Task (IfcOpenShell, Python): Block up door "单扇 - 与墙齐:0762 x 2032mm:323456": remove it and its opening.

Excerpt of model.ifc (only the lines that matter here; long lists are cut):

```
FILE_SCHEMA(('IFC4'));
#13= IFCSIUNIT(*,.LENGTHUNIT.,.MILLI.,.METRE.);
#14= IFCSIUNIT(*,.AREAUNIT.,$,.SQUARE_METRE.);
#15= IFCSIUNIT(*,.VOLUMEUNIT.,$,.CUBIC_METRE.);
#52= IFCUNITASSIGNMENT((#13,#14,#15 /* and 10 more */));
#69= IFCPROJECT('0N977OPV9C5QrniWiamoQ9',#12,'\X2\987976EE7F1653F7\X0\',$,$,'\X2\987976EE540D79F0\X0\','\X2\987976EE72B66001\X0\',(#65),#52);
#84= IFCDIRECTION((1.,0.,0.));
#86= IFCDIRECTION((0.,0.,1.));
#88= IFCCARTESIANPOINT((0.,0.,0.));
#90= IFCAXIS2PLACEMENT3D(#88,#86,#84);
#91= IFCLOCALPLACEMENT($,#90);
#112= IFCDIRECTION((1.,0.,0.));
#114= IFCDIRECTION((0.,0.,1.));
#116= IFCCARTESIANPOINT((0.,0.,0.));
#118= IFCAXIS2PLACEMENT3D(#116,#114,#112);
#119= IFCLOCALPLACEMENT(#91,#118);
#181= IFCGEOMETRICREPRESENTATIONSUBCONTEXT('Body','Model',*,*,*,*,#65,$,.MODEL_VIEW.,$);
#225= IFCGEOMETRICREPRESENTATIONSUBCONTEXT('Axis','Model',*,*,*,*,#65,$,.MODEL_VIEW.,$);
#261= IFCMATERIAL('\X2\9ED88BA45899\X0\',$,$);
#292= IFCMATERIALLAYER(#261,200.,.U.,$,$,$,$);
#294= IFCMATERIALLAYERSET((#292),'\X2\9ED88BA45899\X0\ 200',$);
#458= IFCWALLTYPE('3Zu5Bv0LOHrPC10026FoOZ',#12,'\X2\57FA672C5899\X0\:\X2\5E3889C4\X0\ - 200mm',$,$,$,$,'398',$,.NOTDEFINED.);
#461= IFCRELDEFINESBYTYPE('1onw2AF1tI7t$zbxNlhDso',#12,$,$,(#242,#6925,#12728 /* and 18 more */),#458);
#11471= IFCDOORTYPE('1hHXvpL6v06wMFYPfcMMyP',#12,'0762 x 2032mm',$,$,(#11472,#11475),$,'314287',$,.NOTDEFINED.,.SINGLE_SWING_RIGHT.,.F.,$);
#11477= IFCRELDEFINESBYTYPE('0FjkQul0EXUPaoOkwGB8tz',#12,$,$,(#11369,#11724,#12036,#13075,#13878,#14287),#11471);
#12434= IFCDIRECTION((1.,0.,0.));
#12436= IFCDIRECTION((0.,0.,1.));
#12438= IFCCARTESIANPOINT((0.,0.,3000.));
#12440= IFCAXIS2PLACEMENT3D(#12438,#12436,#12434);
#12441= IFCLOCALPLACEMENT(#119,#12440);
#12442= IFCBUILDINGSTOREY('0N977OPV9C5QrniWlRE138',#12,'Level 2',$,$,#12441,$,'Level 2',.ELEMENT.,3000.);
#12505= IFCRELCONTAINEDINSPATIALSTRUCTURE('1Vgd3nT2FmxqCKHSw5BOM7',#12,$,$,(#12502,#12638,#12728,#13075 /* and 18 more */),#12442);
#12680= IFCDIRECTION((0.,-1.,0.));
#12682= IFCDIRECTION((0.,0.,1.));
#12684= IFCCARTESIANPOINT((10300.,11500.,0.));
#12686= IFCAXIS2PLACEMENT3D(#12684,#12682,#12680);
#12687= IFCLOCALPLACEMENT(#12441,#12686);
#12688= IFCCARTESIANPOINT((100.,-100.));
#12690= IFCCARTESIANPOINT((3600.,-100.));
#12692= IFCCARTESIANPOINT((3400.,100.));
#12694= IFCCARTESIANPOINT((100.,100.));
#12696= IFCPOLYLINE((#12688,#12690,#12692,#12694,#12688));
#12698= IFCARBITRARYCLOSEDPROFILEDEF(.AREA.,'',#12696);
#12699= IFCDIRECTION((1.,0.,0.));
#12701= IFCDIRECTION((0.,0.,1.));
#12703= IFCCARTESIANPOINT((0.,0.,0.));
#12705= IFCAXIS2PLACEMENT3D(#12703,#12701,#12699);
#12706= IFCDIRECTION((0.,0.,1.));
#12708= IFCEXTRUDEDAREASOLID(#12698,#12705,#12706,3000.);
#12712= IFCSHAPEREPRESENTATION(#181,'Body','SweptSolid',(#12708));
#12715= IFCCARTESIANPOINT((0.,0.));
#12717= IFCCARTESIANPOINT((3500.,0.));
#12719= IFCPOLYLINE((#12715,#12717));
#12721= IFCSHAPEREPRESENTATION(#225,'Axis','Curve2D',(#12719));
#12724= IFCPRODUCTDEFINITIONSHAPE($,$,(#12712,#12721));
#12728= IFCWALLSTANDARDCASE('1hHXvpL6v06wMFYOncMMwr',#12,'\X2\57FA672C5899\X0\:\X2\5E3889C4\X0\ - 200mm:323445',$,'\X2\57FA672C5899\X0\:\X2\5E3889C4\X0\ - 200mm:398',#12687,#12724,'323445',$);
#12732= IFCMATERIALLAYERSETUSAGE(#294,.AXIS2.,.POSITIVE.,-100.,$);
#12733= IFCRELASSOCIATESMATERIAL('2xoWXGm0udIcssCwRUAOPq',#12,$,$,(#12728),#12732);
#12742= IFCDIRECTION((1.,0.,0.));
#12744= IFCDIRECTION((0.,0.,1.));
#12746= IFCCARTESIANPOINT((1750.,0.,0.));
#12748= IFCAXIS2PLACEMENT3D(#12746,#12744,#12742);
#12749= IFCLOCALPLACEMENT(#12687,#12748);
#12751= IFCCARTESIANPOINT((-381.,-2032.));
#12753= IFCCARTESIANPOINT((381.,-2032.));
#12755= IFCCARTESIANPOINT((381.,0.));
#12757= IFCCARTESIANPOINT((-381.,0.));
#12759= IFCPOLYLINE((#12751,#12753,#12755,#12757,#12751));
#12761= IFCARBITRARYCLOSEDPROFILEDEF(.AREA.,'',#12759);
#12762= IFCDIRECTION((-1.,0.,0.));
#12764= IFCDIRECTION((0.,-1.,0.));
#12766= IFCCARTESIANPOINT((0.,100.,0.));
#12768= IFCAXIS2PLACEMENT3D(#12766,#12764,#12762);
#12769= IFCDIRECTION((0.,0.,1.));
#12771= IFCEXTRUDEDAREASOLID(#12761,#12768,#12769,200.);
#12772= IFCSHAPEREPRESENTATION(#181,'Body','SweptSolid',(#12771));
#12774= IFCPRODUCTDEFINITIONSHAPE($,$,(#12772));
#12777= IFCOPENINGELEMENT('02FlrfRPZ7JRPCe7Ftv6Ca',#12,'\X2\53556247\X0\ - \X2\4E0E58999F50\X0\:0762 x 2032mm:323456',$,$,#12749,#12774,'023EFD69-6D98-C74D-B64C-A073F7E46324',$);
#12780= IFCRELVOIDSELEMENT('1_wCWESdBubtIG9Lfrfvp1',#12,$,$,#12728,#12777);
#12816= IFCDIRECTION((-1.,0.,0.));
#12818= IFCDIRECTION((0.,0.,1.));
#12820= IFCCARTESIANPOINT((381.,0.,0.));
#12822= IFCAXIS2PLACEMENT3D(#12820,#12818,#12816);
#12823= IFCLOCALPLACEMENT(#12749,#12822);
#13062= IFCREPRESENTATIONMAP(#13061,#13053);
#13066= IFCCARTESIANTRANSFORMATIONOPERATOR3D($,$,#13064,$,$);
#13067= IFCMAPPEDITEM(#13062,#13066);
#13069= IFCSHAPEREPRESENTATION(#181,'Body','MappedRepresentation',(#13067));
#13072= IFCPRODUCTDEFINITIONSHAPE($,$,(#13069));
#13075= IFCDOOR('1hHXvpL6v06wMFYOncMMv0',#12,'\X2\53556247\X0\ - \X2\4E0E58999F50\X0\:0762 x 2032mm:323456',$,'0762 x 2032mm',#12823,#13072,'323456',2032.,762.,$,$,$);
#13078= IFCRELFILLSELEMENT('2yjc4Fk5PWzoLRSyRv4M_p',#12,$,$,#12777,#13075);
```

```python
import ifcopenshell
import ifcopenshell.api.feature
import ifcopenshell.api.root
import ifcopenshell.geom
import ifcopenshell.util.shape

model = ifcopenshell.open("model.ifc")
settings = ifcopenshell.geom.settings()


def volume(element):
    """Net volume in cubic metres, openings subtracted."""
    shape = ifcopenshell.geom.create_shape(settings, element)
    return ifcopenshell.util.shape.get_volume(shape.geometry)


door = model.by_guid("1hHXvpL6v06wMFYOncMMv0")
opening = door.FillsVoids[0].RelatingOpeningElement
wall = opening.VoidsElements[0].RelatingBuildingElement
before = volume(wall)

ifcopenshell.api.root.remove_product(model, product=door)
ifcopenshell.api.feature.remove_feature(model, feature=opening)

after = volume(wall)

print(f"wall volume {before:.3f} -> {after:.3f} m3")

model.write("model-out.ifc")
```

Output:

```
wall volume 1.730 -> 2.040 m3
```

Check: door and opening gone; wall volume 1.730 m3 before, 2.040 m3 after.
